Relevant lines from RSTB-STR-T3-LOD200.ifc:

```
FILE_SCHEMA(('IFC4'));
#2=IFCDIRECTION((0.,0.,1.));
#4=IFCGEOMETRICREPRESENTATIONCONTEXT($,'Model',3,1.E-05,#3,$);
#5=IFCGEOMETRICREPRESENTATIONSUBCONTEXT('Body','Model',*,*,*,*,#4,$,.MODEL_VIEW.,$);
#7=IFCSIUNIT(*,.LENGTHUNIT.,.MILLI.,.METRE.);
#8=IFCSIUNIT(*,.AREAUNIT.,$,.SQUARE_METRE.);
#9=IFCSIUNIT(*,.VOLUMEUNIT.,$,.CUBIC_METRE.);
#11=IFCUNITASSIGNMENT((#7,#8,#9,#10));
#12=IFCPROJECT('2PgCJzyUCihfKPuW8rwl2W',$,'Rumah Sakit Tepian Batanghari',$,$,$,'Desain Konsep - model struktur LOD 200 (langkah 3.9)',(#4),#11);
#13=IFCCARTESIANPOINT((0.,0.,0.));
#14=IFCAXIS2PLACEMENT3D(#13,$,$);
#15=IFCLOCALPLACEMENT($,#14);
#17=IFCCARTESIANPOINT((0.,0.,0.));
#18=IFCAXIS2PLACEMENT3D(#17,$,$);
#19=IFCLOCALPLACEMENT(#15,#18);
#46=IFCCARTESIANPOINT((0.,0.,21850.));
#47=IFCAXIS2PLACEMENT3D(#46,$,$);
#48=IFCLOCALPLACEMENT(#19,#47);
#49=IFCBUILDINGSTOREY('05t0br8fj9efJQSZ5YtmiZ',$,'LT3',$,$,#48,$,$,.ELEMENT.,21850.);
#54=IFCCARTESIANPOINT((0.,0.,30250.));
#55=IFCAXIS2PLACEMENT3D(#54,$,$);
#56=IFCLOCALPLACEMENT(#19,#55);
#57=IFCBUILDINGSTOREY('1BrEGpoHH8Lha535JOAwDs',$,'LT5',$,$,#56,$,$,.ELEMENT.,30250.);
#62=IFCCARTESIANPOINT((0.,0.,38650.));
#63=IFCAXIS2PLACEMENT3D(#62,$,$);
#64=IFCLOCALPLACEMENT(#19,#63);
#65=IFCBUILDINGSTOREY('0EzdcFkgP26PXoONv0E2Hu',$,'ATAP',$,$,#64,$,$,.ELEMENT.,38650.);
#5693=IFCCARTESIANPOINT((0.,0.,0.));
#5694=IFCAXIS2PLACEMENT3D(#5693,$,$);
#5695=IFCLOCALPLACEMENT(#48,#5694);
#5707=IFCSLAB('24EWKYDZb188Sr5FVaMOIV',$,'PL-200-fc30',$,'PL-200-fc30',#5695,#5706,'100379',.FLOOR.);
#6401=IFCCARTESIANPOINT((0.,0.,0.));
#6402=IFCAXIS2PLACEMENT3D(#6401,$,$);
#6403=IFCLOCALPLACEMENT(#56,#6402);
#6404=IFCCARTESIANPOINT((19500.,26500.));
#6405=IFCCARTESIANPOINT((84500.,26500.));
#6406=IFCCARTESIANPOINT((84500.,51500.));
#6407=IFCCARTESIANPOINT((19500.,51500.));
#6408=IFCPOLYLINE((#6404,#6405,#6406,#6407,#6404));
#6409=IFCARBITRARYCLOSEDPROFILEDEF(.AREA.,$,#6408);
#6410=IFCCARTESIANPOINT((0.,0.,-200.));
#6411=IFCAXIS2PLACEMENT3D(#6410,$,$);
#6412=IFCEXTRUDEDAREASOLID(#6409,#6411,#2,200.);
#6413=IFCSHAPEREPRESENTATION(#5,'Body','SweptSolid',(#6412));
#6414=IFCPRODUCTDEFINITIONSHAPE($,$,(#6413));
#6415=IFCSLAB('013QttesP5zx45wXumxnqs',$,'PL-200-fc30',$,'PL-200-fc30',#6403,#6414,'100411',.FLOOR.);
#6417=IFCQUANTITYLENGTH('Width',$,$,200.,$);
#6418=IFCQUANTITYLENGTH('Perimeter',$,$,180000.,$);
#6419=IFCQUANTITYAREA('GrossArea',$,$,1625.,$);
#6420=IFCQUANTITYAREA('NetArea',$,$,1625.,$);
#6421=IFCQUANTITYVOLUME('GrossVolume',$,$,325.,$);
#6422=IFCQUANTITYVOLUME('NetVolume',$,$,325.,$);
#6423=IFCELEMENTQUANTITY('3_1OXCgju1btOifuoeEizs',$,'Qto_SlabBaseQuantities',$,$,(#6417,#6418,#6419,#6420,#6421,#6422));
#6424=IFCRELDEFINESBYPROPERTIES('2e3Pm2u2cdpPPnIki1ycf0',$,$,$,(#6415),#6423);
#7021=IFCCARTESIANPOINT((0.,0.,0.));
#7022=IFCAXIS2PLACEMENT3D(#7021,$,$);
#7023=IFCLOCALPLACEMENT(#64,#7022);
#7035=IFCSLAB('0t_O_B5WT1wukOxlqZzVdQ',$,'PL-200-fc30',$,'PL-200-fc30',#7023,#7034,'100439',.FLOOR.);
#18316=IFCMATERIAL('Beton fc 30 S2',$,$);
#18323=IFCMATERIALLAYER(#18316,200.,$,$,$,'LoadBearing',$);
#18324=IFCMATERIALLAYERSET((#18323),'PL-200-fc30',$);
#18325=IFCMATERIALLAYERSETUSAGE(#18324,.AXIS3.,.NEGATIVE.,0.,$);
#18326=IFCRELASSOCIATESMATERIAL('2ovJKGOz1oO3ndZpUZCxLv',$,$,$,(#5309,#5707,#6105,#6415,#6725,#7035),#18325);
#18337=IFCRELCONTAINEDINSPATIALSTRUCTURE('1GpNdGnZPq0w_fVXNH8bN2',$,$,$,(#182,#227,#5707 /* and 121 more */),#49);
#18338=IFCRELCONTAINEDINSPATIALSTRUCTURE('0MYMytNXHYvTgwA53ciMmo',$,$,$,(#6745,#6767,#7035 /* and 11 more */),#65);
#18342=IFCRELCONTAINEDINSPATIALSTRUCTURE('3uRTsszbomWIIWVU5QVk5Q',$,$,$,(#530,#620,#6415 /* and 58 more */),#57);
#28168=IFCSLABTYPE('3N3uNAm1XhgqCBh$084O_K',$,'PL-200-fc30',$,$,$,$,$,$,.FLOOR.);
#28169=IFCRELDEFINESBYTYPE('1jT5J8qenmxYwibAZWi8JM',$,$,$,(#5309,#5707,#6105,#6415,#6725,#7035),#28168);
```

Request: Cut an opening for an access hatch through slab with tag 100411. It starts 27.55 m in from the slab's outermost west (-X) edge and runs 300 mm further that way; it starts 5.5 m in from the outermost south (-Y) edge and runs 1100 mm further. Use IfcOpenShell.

```python
import numpy as np
import ifcopenshell
import ifcopenshell.api.feature
import ifcopenshell.api.geometry
import ifcopenshell.api.pset
import ifcopenshell.api.root
import ifcopenshell.geom
import ifcopenshell.util.element
import ifcopenshell.util.placement
import ifcopenshell.util.representation
import ifcopenshell.util.shape
import ifcopenshell.util.unit

model = ifcopenshell.open("RSTB-STR-T3-LOD200.ifc")
unit_scale = ifcopenshell.util.unit.calculate_unit_scale(model)
area_scale = ifcopenshell.util.unit.calculate_unit_scale(model, "AREAUNIT")
volume_scale = ifcopenshell.util.unit.calculate_unit_scale(model, "VOLUMEUNIT")
settings = ifcopenshell.geom.settings()


def volume(element):
    """Net volume in cubic metres, openings subtracted."""
    shape = ifcopenshell.geom.create_shape(settings, element)
    return ifcopenshell.util.shape.get_volume(shape.geometry)


slab = model.by_id(6415)
before = volume(slab)

# Extent in the slab's own axes, in metres. The edges named are its -X and -Y sides.
slab_shape = ifcopenshell.geom.create_shape(settings, slab)
vertices = ifcopenshell.util.shape.get_vertices(slab_shape.geometry)
x_min, y_min, bottom = vertices.min(axis=0)
top = vertices[:, 2].max()

opening = ifcopenshell.api.root.create_entity(model, ifc_class="IfcOpeningElement", name="Access hatch opening", predefined_type="OPENING")
context = ifcopenshell.util.representation.get_context(model, "Model", "Body", "MODEL_VIEW")
width, depth = 0.3, 1.1
outline = [(0.0, 0.0), (width, 0.0), (width, depth), (0.0, depth), (0.0, 0.0)]
# Overshoot both faces by 50 mm so the cut is clean.
shape = ifcopenshell.api.geometry.add_slab_representation(
    model, context=context, depth=top - bottom + 0.1, polyline=outline
)
ifcopenshell.api.geometry.assign_representation(model, product=opening, representation=shape)

matrix = ifcopenshell.util.placement.get_local_placement(slab.ObjectPlacement)
matrix[:, 3] = matrix @ np.append(np.array([x_min + 27.55, y_min + 5.5, bottom - 0.05]) / unit_scale, 1.0)
ifcopenshell.api.geometry.edit_object_placement(model, product=opening, matrix=matrix, is_si=False)
ifcopenshell.api.feature.add_feature(model, feature=opening, element=slab)

after = volume(slab)

# Update the slab's stored quantities.
qto = model.by_id(ifcopenshell.util.element.get_pset(slab, "Qto_SlabBaseQuantities", should_inherit=False)["id"])
ifcopenshell.api.pset.edit_qto(model, qto=qto, properties={
    "NetArea": after / (top - bottom) / area_scale,
    "NetVolume": after / volume_scale,
})

print(f"slab volume {before:.3f} -> {after:.3f} m3")

model.write("RSTB-STR-T3-LOD200-out.ifc")
```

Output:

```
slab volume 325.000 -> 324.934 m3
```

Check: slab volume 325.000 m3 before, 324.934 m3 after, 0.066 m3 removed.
